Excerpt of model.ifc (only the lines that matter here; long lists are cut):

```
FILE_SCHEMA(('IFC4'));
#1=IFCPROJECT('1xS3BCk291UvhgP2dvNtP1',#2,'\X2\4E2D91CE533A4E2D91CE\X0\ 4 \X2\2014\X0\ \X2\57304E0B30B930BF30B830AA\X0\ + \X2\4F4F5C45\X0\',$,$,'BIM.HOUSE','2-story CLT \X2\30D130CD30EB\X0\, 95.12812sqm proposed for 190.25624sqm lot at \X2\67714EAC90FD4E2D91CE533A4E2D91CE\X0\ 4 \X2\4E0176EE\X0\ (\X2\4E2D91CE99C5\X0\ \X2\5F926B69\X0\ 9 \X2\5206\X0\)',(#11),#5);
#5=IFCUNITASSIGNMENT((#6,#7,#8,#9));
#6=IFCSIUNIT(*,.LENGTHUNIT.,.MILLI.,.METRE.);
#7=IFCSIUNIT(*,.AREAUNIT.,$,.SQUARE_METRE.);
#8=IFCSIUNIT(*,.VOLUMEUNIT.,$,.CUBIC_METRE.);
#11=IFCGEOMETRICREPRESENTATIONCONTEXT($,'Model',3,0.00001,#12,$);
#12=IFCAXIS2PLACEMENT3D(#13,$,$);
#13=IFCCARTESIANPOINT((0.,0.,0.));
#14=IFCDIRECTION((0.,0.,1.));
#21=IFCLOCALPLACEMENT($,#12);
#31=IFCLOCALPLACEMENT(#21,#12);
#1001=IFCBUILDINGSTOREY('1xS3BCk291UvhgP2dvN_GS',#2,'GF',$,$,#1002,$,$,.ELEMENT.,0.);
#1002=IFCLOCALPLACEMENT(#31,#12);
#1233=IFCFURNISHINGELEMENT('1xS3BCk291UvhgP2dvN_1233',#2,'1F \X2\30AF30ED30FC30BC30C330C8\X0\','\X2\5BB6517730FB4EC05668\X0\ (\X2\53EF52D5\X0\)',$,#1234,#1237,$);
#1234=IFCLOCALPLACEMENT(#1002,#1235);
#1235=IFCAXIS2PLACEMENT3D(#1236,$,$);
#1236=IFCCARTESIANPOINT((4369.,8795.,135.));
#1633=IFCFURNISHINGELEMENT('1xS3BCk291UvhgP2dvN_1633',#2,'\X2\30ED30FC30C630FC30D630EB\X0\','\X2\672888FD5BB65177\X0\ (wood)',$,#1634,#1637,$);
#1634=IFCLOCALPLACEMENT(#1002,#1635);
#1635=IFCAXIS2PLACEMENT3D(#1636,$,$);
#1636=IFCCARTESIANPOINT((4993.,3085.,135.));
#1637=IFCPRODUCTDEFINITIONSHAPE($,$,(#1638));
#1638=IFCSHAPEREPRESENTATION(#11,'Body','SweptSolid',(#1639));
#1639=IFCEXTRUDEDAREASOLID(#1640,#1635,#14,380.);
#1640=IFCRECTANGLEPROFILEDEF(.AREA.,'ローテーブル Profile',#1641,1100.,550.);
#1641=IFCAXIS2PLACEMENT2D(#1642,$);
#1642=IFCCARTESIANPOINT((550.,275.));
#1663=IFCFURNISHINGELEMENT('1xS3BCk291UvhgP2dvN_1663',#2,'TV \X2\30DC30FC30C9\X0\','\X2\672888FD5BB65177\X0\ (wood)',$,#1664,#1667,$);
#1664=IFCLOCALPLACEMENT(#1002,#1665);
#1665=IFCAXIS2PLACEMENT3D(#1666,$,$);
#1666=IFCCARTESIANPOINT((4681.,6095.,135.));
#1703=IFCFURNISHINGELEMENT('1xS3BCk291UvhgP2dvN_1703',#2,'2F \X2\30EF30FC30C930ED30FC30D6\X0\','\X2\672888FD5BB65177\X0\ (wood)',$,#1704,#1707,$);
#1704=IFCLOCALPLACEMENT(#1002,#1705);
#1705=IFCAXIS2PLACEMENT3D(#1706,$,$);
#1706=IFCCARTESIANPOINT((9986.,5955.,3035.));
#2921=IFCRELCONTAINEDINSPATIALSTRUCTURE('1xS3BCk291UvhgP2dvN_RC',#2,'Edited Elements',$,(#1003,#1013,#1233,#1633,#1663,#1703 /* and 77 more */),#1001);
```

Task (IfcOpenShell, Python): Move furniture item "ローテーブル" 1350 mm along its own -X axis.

```python
import ifcopenshell
import ifcopenshell.api.geometry
import ifcopenshell.util.placement
import ifcopenshell.util.unit

model = ifcopenshell.open("model.ifc")
unit_scale = ifcopenshell.util.unit.calculate_unit_scale(model)

item = model.by_id(1633)
matrix = ifcopenshell.util.placement.get_local_placement(item.ObjectPlacement)
matrix[:3, 3] -= matrix[:3, 0] * 1.35 / unit_scale
ifcopenshell.api.geometry.edit_object_placement(model, product=item, matrix=matrix, is_si=False)

print(ifcopenshell.util.placement.get_local_placement(item.ObjectPlacement).round(3) + 0.0)

model.write("model_edited.ifc")
```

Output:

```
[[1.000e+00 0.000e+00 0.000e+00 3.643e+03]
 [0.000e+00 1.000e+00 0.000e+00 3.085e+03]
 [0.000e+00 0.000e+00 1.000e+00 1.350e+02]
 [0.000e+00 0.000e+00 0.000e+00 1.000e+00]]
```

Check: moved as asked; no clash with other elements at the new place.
